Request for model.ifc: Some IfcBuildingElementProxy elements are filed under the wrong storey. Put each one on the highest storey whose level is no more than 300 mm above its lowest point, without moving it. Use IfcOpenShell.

First a look at what the model holds.

```python
import ifcopenshell
import ifcopenshell.util.element
import ifcopenshell.util.placement

model = ifcopenshell.open("model.ifc")
print(model.schema)
for storey in model.by_type("IfcBuildingStorey"):
    level = ifcopenshell.util.placement.get_storey_elevation(storey)
    count = sum(e.is_a("IfcBuildingElementProxy") for e in ifcopenshell.util.element.get_contained(storey))
    print(storey.id(), storey.Name, round(level, 3), count, sep=" | ")
```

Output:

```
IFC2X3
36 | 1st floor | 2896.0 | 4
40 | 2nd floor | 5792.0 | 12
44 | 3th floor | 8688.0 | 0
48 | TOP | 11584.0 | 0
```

```python
import ifcopenshell
import ifcopenshell.api.spatial
import ifcopenshell.geom
import ifcopenshell.util.element
import ifcopenshell.util.placement
import ifcopenshell.util.shape
import ifcopenshell.util.unit

model = ifcopenshell.open("model.ifc")
unit_scale = ifcopenshell.util.unit.calculate_unit_scale(model)
settings = ifcopenshell.geom.settings()

levels = sorted(
    ((ifcopenshell.util.placement.get_storey_elevation(s) * unit_scale, s) for s in model.by_type("IfcBuildingStorey")),
    key=lambda pair: pair[0],
)

for e in model.by_type("IfcBuildingElementProxy"):
    current = e.ContainedInStructure[0].RelatingStructure if e.ContainedInStructure else None
    if current is None or not current.is_a("IfcBuildingStorey"):
        continue
    shape = ifcopenshell.geom.create_shape(settings, e)
    bottom = ifcopenshell.util.shape.get_shape_bottom_elevation(shape, shape.geometry)
    below = [s for level, s in levels if level <= bottom + 0.3]
    storey = below[-1] if below else levels[0][1]
    if storey != current:
        # assign_container keeps the world position.
        ifcopenshell.api.spatial.assign_container(model, products=[e], relating_structure=storey)
        print(e.id(), current.Name, "->", storey.Name)

model.write("model_rev.ifc")
```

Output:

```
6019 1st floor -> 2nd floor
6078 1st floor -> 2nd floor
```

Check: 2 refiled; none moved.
